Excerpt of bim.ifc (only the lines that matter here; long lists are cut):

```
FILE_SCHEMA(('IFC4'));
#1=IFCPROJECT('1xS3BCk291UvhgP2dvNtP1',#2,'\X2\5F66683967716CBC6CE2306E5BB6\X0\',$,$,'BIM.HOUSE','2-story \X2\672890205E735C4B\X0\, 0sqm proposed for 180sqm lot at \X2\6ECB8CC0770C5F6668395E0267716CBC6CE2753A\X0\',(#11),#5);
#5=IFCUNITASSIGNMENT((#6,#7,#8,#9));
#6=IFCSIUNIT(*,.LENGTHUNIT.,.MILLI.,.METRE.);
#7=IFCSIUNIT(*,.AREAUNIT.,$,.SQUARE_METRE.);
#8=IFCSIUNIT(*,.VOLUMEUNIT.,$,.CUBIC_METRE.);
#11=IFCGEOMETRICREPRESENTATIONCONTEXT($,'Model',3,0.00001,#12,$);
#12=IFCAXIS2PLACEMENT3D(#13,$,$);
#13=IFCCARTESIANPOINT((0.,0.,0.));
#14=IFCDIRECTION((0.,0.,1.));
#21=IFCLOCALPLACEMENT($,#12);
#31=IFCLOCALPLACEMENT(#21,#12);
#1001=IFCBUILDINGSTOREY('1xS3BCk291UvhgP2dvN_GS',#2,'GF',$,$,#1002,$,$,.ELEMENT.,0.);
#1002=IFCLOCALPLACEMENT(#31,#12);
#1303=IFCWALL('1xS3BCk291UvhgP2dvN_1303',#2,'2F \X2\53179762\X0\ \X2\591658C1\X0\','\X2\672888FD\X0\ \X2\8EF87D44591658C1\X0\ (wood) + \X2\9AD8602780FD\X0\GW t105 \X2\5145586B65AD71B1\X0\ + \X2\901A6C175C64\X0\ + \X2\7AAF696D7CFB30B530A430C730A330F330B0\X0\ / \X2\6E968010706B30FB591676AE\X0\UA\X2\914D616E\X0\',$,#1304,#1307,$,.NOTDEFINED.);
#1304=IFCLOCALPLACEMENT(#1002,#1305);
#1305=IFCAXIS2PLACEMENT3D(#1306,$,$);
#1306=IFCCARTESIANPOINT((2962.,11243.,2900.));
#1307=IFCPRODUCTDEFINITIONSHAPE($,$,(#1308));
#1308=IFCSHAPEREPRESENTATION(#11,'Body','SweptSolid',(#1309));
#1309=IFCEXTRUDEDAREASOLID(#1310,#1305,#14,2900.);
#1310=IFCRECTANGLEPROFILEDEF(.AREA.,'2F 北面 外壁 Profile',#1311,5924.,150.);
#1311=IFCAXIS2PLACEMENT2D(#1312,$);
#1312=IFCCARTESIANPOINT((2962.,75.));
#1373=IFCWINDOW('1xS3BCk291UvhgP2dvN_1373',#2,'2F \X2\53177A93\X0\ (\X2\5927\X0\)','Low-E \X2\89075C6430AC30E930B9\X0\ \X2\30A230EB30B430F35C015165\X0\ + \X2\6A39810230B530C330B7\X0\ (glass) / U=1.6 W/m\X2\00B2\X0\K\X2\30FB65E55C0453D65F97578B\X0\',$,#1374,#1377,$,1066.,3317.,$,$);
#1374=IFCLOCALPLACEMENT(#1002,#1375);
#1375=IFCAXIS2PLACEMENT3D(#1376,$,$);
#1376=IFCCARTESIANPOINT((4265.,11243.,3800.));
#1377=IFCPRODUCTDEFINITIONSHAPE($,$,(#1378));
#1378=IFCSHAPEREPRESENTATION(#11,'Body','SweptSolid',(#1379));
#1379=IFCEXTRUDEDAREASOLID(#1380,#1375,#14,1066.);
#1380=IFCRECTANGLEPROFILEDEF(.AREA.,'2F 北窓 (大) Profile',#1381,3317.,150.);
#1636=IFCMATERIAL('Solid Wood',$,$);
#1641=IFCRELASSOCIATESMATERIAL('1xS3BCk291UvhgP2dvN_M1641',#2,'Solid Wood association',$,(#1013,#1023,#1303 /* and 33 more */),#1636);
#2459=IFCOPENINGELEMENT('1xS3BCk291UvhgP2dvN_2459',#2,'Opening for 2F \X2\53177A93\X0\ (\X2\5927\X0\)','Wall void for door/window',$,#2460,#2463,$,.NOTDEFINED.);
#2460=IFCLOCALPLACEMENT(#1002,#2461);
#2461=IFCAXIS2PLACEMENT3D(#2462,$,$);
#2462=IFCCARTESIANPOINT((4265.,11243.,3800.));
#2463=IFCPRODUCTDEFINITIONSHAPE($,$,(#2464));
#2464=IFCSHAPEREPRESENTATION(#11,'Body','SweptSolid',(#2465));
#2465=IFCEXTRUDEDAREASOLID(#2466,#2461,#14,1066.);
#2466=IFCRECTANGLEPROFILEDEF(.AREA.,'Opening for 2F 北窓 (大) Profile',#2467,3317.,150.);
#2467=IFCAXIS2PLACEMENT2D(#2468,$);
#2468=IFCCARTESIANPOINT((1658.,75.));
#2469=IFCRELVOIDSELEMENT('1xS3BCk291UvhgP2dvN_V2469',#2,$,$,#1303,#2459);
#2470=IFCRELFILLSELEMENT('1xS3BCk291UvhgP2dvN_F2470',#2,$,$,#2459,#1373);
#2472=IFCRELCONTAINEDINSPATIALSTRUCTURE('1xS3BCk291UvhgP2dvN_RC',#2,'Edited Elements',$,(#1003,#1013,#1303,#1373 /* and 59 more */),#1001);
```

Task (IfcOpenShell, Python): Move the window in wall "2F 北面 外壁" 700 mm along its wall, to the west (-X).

```python
import ifcopenshell
import ifcopenshell.api.geometry
import ifcopenshell.util.placement
import ifcopenshell.util.unit

model = ifcopenshell.open("bim.ifc")
unit_scale = ifcopenshell.util.unit.calculate_unit_scale(model)

window = model.by_guid("1xS3BCk291UvhgP2dvN_1373")
opening = window.FillsVoids[0].RelatingOpeningElement
wall = opening.VoidsElements[0].RelatingBuildingElement

wall_matrix = ifcopenshell.util.placement.get_local_placement(wall.ObjectPlacement)
shift = wall_matrix[:3, 0] * -0.7 / unit_scale
before = ifcopenshell.util.placement.get_local_placement(window.ObjectPlacement)[:3, 3].copy()

# The window is not placed relative to its opening, so move both.
for product in (opening, window):
    matrix = ifcopenshell.util.placement.get_local_placement(product.ObjectPlacement)
    matrix[:3, 3] += shift
    ifcopenshell.api.geometry.edit_object_placement(model, product=product, matrix=matrix, is_si=False)

after = ifcopenshell.util.placement.get_local_placement(window.ObjectPlacement)[:3, 3]
print("window moved by", (after - before).round(3) + 0.0)

model.write("bim_updated.ifc")
```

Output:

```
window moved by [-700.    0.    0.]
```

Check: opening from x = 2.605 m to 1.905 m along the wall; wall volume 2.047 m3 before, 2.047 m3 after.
